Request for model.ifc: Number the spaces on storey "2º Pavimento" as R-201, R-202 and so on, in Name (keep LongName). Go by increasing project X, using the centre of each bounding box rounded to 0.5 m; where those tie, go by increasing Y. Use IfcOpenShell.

First a look at what the model holds.

```python
import ifcopenshell
import ifcopenshell.util.element
import ifcopenshell.util.placement

model = ifcopenshell.open("model.ifc")
print(model.schema)
storey = next(s for s in model.by_type("IfcBuildingStorey") if s.Name == "2º Pavimento")
spaces = [e for e in ifcopenshell.util.element.get_decomposition(storey) if e.is_a("IfcSpace")]
for e in sorted(spaces, key=lambda e: e.id()):
    origin = ifcopenshell.util.placement.get_local_placement(e.ObjectPlacement)[:3, 3]
    print(e.id(), e.Name, e.LongName, origin.round(2) + 0.0, sep=" | ")
```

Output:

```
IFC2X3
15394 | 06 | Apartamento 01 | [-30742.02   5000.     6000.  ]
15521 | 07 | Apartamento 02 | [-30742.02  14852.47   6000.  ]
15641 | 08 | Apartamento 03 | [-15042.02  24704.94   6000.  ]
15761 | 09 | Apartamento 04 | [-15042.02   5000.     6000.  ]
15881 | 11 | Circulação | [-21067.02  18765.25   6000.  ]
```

```python
import ifcopenshell
import ifcopenshell.geom
import ifcopenshell.util.element
import ifcopenshell.util.shape

model = ifcopenshell.open("model.ifc")
settings = ifcopenshell.geom.settings()
settings.set("use-world-coords", True)


def centre(element):
    shape = ifcopenshell.geom.create_shape(settings, element)
    return ifcopenshell.util.shape.get_bbox_centroid(shape.geometry)


storey = next(s for s in model.by_type("IfcBuildingStorey") if s.Name == "2º Pavimento")
spaces = [e for e in ifcopenshell.util.element.get_decomposition(storey) if e.is_a("IfcSpace")]

# Insertion points can sit at a corner or the storey origin, so sort by the geometry (in metres).
centres = {e: centre(e) for e in spaces}
spaces.sort(key=lambda e: (round(centres[e][0] / 0.5), centres[e][1]))

for i, e in enumerate(spaces, start=1):
    number = f"R-2{i:02d}"
    e.Name = number
    print(e.id(), number)

model.write("model-out.ifc")
```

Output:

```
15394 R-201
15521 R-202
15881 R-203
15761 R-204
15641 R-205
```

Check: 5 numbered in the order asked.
